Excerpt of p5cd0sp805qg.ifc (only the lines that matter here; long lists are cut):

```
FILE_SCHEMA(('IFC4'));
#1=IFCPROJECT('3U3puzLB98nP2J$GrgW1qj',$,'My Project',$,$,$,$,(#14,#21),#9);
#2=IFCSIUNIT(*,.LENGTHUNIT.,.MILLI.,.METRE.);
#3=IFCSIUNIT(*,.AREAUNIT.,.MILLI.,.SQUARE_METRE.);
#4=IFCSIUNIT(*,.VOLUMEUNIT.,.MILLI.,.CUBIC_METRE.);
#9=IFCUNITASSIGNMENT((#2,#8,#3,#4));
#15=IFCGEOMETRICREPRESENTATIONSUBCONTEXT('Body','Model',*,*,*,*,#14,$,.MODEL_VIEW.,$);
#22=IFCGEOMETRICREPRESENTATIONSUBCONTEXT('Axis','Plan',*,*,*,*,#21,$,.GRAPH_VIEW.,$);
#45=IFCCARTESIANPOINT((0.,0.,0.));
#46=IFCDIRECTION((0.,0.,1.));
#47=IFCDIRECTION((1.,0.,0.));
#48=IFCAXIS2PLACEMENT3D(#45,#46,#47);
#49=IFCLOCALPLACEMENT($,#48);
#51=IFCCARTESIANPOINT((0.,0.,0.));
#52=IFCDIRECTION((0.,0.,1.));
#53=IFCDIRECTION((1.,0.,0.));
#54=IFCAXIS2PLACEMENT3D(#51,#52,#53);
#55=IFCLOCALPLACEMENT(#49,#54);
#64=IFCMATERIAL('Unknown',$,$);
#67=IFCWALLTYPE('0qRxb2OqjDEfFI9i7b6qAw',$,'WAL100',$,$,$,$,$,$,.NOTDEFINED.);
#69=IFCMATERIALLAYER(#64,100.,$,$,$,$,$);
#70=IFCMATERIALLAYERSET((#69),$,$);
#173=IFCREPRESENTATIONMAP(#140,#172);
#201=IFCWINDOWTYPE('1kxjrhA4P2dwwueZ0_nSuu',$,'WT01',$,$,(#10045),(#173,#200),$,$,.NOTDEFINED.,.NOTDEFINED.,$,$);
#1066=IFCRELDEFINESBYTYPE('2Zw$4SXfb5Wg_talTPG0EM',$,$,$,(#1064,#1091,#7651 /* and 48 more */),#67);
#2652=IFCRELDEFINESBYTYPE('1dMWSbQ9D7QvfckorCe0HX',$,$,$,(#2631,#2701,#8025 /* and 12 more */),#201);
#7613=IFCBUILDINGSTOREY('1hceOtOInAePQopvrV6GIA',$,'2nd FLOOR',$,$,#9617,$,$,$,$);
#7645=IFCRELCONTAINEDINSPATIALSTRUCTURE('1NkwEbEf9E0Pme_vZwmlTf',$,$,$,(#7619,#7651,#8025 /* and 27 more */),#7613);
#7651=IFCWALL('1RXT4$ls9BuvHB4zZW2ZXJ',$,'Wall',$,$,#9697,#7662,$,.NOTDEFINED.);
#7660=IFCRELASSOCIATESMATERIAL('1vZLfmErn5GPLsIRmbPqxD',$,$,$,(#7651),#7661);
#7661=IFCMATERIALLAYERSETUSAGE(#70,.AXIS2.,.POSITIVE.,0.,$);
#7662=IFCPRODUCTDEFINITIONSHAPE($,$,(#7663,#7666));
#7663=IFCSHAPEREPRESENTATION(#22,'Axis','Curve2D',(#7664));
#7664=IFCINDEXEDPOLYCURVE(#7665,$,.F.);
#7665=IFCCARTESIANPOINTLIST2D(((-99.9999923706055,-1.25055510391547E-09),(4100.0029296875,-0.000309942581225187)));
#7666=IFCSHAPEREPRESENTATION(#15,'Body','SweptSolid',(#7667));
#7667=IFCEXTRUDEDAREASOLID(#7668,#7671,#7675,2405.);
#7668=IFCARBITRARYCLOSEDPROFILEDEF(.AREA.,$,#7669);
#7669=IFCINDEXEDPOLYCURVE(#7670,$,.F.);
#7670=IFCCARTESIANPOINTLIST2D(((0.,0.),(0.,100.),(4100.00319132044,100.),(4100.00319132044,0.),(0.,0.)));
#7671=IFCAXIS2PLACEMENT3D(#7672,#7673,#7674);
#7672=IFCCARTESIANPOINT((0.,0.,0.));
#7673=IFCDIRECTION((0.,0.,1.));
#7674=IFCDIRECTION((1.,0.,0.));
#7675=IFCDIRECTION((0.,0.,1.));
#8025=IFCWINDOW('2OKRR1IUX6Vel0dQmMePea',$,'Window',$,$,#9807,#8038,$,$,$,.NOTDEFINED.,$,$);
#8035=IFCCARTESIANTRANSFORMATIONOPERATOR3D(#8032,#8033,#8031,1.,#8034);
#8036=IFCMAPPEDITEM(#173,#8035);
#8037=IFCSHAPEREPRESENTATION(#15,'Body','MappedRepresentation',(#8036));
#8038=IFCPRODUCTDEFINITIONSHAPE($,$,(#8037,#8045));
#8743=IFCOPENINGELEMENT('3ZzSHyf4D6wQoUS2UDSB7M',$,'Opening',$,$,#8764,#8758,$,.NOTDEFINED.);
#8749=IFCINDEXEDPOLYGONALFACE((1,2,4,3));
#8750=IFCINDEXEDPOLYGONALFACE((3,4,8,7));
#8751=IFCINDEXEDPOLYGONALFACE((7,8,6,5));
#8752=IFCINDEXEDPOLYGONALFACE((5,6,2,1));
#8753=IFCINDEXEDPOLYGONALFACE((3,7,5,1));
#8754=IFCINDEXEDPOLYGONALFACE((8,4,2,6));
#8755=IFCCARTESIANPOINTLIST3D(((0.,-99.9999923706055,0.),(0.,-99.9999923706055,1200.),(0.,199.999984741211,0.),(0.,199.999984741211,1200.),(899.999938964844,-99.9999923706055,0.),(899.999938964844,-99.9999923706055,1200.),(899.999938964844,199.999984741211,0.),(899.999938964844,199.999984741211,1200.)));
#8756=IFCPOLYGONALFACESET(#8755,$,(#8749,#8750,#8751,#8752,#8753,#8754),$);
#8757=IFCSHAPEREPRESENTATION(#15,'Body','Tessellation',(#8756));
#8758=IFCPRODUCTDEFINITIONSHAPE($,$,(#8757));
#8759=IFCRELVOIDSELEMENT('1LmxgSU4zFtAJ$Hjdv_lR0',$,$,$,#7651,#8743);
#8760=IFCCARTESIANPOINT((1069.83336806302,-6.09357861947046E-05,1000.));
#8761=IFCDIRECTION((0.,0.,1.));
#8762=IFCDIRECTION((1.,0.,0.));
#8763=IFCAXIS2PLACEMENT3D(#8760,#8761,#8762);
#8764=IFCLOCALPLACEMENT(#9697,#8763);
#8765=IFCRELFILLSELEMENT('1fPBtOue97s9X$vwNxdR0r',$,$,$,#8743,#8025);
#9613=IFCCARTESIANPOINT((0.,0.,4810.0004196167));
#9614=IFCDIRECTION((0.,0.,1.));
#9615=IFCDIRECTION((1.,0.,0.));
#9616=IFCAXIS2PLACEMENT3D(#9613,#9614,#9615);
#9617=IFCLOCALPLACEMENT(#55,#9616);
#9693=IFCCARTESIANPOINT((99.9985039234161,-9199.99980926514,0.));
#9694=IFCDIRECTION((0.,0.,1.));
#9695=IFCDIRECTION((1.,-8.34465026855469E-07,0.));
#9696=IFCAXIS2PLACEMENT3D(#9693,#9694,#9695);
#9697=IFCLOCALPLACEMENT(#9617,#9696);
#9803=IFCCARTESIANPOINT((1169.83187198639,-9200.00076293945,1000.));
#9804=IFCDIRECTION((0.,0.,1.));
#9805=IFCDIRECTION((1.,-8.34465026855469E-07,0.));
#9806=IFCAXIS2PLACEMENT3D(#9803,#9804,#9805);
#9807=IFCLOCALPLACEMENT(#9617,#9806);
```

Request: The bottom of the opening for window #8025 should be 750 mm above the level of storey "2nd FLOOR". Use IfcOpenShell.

```python
import numpy as np
import ifcopenshell
import ifcopenshell.api.geometry
import ifcopenshell.geom
import ifcopenshell.util.element
import ifcopenshell.util.placement
import ifcopenshell.util.shape
import ifcopenshell.util.unit

model = ifcopenshell.open("p5cd0sp805qg.ifc")
unit_scale = ifcopenshell.util.unit.calculate_unit_scale(model)

window = model.by_id(8025)
opening = window.FillsVoids[0].RelatingOpeningElement
storey = ifcopenshell.util.element.get_container(window, ifc_class="IfcBuildingStorey")
level = ifcopenshell.util.placement.get_local_placement(storey.ObjectPlacement)[2, 3]

# The opening's origin need not be at the sill, so measure its lowest point.
shape = ifcopenshell.geom.create_shape(ifcopenshell.geom.settings(), opening)
bottom = ifcopenshell.util.shape.get_shape_bottom_elevation(shape, shape.geometry) / unit_scale
dz = level + 750.0 - bottom

shift = np.array([0.0, 0.0, dz])
# The window is not placed relative to its opening, so move both.
for product in (opening, window):
    matrix = ifcopenshell.util.placement.get_local_placement(product.ObjectPlacement)
    matrix[:3, 3] += shift
    ifcopenshell.api.geometry.edit_object_placement(model, product=product, matrix=matrix, is_si=False)

print(f"moved by {dz * unit_scale:+.3f} m")

model.write("p5cd0sp805qg_rev.ifc")
```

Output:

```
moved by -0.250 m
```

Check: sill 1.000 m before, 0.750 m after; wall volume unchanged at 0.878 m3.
